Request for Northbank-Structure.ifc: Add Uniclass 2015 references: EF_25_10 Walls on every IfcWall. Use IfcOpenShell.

First a look at what the model holds.

```python
import ifcopenshell

model = ifcopenshell.open("Northbank-Structure.ifc")
print(model.schema)
print("classifications:", [c.Name for c in model.by_type("IfcClassification")])
for ifc_class in ("IfcDoor", "IfcRoof", "IfcStair", "IfcWall", "IfcWindow"):
    print(ifc_class, len(model.by_type(ifc_class)))
```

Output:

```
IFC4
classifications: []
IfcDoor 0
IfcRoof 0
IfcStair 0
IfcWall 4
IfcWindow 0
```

```python
import ifcopenshell
import ifcopenshell.api.classification

model = ifcopenshell.open("Northbank-Structure.ifc")

system = ifcopenshell.api.classification.add_classification(model, classification="Uniclass 2015")

codes = {
    "IfcWall": ("EF_25_10", "Walls"),
}
for ifc_class, (code, name) in codes.items():
    products = model.by_type(ifc_class)
    ifcopenshell.api.classification.add_reference(
        model, products=products, classification=system, identification=code, name=name
    )
    print(code, len(products))

model.write("Northbank-Structure-out.ifc")
```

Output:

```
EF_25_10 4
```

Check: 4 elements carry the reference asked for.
